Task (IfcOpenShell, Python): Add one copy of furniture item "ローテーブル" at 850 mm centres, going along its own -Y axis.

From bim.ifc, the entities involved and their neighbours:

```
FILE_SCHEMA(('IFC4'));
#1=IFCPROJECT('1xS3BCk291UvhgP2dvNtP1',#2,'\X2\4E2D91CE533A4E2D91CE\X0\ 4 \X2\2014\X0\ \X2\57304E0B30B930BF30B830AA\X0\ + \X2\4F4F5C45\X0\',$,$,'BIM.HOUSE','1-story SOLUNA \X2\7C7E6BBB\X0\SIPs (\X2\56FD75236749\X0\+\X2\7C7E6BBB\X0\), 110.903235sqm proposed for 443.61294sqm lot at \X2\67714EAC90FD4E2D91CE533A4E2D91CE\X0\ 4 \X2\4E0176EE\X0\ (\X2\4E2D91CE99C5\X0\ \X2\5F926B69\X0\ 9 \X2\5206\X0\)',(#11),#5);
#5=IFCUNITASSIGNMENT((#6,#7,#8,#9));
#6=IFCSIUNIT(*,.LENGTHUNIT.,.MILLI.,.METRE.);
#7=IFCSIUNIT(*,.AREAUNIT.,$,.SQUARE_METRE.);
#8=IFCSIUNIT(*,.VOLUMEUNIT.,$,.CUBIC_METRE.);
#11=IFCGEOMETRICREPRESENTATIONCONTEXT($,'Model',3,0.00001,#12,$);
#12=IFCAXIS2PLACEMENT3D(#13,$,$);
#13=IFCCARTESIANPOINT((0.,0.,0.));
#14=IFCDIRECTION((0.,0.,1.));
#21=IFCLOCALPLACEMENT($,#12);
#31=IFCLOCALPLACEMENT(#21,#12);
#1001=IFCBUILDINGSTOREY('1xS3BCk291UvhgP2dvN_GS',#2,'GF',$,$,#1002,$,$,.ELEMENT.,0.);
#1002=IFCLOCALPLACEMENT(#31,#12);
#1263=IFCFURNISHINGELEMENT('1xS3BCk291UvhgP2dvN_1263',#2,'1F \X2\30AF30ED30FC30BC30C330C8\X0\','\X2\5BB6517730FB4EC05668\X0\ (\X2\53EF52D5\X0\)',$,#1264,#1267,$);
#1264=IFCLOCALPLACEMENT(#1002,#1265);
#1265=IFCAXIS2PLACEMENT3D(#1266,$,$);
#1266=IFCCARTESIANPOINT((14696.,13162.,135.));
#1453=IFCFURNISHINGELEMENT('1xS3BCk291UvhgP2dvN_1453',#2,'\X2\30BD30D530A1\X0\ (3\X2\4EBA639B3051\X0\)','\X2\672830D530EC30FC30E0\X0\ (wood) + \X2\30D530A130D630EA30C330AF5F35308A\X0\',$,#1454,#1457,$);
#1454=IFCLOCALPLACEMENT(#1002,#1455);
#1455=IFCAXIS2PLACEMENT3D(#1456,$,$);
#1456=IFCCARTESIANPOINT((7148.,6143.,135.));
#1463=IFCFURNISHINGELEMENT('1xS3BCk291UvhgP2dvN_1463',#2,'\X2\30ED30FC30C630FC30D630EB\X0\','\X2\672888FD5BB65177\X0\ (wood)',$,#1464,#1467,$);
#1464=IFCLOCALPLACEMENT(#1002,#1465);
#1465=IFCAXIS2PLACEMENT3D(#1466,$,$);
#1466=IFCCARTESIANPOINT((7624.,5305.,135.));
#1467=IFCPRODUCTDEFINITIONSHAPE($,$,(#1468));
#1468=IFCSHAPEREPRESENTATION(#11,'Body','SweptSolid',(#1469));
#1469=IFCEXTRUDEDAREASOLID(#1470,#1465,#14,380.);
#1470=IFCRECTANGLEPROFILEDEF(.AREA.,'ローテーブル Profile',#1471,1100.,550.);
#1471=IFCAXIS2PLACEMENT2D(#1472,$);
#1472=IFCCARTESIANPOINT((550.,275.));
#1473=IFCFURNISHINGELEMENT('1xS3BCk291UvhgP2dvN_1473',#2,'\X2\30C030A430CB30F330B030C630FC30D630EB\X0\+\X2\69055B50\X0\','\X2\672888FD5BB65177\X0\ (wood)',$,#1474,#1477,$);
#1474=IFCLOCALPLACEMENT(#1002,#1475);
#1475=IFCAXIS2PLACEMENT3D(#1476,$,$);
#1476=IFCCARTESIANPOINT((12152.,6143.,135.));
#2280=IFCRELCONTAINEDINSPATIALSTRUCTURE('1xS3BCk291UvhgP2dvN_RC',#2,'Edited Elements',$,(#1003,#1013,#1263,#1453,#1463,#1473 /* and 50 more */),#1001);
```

```python
import ifcopenshell
import ifcopenshell.api.geometry
import ifcopenshell.api.root
import ifcopenshell.util.element
import ifcopenshell.util.placement
import ifcopenshell.util.unit

model = ifcopenshell.open("bim.ifc")
unit_scale = ifcopenshell.util.unit.calculate_unit_scale(model)


def reuse_history(source, copy):
    """copy_class also copies each property set's owner history, people and application; keep the originals."""
    for rel in copy.IsDefinedBy:
        if rel.is_a("IfcRelDefinesByProperties") and (history := rel.RelatingPropertyDefinition.OwnerHistory):
            rel.RelatingPropertyDefinition.OwnerHistory = source.OwnerHistory
            ifcopenshell.util.element.remove_deep2(model, history)


source = model.by_guid("1xS3BCk291UvhgP2dvN_1463")
base = ifcopenshell.util.placement.get_local_placement(source.ObjectPlacement)
step = -base[:3, 1] * 0.85 / unit_scale

for i in range(1, 2):
    copy = ifcopenshell.api.root.copy_class(model, product=source)
    copy.Representation = ifcopenshell.util.element.copy_deep(
        model, source.Representation, exclude=["IfcGeometricRepresentationContext", "IfcRepresentationMap"]
    )
    reuse_history(source, copy)
    matrix = base.copy()
    matrix[:3, 3] += i * step
    print("added at", matrix[:3, 3].round(3) + 0.0)
    ifcopenshell.api.geometry.edit_object_placement(model, product=copy, matrix=matrix, is_si=False)

model.write("bim-out.ifc")
```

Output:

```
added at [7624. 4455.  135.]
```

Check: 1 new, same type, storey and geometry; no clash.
